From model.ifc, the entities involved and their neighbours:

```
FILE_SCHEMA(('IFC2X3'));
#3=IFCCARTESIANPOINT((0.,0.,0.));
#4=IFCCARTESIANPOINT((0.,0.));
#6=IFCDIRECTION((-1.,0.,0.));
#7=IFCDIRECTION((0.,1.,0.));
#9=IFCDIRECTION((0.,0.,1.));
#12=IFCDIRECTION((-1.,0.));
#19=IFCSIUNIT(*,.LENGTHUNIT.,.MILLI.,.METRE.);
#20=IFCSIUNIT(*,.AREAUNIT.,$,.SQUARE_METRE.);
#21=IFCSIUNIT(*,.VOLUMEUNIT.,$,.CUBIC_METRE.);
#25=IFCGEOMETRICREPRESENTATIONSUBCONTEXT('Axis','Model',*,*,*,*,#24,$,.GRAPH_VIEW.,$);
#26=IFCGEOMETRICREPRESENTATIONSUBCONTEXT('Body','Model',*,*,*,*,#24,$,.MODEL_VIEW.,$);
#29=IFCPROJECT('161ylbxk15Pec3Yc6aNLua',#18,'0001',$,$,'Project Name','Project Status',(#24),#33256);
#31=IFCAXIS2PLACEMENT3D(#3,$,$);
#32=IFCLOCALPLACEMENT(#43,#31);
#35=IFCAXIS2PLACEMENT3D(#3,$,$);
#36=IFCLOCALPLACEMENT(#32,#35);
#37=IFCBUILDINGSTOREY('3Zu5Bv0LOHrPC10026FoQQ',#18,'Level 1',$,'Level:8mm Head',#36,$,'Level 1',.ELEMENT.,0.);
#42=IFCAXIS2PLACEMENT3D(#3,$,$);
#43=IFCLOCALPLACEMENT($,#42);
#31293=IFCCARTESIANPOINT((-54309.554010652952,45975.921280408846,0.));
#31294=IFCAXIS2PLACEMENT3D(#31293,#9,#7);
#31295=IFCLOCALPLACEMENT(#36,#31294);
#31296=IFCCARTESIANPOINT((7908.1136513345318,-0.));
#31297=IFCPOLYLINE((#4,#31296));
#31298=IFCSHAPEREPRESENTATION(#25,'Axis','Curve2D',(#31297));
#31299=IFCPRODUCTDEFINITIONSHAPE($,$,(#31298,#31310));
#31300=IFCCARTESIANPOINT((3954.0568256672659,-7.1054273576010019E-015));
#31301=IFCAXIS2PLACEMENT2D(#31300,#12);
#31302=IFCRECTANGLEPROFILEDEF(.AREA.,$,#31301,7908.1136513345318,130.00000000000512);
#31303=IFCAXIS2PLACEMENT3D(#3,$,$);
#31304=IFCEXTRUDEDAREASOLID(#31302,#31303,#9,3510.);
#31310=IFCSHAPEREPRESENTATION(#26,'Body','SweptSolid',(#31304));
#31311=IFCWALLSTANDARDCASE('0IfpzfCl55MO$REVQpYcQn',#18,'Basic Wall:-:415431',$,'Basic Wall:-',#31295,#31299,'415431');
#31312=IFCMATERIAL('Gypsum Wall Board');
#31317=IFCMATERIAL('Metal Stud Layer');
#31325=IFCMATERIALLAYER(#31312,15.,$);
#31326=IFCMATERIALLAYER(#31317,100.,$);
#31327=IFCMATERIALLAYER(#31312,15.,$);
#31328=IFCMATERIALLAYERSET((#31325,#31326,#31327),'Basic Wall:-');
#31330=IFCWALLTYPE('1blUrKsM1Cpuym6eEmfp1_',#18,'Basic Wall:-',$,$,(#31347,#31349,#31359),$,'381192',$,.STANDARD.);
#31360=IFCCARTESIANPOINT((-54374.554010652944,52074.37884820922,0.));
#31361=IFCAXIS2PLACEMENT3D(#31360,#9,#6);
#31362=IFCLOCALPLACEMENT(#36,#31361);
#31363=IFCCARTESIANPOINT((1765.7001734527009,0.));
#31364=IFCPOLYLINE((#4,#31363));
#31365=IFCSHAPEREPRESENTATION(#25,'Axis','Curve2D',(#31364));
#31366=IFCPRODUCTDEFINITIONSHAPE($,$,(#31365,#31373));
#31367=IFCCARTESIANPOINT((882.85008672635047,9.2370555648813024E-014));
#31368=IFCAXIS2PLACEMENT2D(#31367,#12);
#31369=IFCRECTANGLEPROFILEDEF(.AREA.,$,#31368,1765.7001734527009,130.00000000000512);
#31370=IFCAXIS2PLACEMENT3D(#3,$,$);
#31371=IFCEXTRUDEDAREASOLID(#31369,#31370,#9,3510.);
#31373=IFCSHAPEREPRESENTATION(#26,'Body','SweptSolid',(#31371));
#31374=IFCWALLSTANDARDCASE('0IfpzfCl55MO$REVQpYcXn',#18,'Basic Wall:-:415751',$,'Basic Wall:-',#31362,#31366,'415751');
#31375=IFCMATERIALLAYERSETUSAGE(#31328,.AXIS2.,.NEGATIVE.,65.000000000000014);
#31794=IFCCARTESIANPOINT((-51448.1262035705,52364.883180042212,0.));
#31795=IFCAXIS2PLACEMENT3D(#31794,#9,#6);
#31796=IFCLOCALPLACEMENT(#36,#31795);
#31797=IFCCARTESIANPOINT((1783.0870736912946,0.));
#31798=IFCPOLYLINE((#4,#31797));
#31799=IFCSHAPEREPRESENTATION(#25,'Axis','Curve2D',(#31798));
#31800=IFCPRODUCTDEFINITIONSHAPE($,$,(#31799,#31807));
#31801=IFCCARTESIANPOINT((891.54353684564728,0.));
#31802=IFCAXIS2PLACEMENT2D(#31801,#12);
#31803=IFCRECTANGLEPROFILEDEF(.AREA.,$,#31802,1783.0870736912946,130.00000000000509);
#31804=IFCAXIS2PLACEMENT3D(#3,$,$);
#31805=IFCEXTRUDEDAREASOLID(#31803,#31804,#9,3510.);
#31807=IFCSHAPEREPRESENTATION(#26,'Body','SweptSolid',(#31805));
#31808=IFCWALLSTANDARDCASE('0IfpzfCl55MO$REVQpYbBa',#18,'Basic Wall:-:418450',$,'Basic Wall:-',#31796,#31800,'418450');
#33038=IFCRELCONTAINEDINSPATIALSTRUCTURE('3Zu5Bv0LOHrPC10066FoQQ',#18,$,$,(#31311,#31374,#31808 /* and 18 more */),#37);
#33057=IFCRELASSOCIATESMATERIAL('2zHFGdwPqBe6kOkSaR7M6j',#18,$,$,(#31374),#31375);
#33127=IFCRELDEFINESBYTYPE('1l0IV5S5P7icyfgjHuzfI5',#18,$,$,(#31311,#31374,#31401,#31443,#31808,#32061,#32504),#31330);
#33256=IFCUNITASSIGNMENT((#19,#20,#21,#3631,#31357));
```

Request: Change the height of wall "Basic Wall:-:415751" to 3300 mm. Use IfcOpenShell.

```python
import ifcopenshell
import ifcopenshell.geom
import ifcopenshell.util.representation
import ifcopenshell.util.shape

model = ifcopenshell.open("model.ifc")
settings = ifcopenshell.geom.settings()


def volume(element):
    """Net volume in cubic metres, openings subtracted."""
    shape = ifcopenshell.geom.create_shape(settings, element)
    return ifcopenshell.util.shape.get_volume(shape.geometry)


wall = model.by_guid("0IfpzfCl55MO$REVQpYcXn")
before = volume(wall)

body = ifcopenshell.util.representation.get_representation(wall, "Model", "Body")
solid = body.Items[0]
old_height = solid.Depth
solid.Depth = 3300.0
after = volume(wall)

print(f"height {old_height:g} -> {solid.Depth:g}, volume {before:.3f} -> {after:.3f} m3")

model.write("model_edited.ifc")
```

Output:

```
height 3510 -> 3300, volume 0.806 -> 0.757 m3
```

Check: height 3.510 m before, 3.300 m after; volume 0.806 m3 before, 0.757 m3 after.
